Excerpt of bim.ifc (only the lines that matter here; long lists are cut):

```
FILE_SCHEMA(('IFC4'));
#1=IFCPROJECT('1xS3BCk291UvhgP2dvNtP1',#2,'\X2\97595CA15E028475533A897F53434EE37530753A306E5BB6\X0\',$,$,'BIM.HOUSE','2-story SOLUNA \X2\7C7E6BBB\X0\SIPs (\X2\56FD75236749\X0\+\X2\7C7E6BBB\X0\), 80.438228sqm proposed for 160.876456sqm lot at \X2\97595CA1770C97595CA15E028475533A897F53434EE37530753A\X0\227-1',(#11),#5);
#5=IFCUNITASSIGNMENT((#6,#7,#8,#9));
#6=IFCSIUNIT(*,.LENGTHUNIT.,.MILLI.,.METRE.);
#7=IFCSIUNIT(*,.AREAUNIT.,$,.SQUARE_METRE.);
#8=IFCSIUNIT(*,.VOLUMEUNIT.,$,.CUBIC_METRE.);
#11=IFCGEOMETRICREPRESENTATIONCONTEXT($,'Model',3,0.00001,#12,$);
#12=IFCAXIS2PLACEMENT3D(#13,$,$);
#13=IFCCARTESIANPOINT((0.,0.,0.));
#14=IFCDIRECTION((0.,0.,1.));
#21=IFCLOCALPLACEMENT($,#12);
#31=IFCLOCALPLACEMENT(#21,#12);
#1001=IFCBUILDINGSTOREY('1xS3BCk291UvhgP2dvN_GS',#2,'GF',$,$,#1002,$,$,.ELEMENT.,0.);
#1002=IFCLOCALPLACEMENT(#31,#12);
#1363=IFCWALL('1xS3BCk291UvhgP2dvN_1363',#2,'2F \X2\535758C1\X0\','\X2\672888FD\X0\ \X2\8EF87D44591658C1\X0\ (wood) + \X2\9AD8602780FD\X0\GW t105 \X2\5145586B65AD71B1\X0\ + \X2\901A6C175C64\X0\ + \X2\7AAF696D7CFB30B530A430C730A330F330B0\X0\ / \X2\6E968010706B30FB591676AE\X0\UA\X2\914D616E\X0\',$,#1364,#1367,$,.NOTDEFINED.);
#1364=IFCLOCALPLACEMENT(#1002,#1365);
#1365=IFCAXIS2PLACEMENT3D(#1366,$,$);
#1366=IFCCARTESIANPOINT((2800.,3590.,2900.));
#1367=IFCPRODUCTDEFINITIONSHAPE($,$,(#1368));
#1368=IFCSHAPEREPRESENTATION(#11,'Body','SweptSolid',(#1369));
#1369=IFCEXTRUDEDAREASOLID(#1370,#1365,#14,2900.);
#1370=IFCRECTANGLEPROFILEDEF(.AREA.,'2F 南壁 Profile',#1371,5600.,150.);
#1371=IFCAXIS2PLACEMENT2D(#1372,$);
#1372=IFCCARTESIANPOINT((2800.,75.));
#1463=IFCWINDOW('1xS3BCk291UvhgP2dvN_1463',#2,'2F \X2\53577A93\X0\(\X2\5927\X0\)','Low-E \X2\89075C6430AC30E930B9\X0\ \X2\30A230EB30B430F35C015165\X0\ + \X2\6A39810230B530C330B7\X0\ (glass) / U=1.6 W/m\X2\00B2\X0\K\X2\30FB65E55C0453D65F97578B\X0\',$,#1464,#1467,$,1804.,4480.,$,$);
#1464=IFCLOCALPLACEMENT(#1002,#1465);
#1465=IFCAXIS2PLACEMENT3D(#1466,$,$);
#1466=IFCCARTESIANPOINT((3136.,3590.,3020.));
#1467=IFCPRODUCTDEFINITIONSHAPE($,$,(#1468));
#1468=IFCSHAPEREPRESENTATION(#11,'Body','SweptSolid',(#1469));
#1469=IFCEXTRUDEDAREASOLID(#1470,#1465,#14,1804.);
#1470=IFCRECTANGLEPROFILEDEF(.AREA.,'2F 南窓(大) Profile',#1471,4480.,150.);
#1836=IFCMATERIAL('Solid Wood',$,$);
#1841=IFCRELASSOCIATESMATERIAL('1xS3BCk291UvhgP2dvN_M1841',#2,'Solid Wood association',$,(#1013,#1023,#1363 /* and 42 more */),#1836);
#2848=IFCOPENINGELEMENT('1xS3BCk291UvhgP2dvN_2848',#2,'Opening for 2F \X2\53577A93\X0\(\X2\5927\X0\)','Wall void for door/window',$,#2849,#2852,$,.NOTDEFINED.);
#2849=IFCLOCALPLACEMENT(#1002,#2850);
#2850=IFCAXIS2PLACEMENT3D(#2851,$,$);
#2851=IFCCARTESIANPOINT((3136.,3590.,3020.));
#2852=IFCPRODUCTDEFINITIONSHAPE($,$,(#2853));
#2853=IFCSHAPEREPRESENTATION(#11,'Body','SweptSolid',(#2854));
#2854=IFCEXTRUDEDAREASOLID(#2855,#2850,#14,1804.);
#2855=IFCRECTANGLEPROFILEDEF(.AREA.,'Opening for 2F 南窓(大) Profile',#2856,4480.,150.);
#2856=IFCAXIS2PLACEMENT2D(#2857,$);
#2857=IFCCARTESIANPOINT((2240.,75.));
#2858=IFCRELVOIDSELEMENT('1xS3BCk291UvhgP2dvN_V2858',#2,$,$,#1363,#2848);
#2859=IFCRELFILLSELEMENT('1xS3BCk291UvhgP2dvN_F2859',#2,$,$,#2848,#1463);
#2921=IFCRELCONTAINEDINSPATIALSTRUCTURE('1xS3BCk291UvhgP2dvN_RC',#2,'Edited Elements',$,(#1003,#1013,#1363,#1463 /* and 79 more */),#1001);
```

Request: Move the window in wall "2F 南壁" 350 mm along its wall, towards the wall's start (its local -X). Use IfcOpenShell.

```python
import ifcopenshell
import ifcopenshell.api.geometry
import ifcopenshell.util.placement

model = ifcopenshell.open("bim.ifc")

window = model.by_id(1463)
opening = window.FillsVoids[0].RelatingOpeningElement
wall = opening.VoidsElements[0].RelatingBuildingElement

wall_matrix = ifcopenshell.util.placement.get_local_placement(wall.ObjectPlacement)
shift = wall_matrix[:3, 0] * -350.0
before = ifcopenshell.util.placement.get_local_placement(window.ObjectPlacement)[:3, 3].copy()

# The window is not placed relative to its opening, so move both.
for product in (opening, window):
    matrix = ifcopenshell.util.placement.get_local_placement(product.ObjectPlacement)
    matrix[:3, 3] += shift
    ifcopenshell.api.geometry.edit_object_placement(model, product=product, matrix=matrix, is_si=False)

after = ifcopenshell.util.placement.get_local_placement(window.ObjectPlacement)[:3, 3]
print("window moved by", (after - before).round(3) + 0.0)

model.write("bim_rev.ifc")
```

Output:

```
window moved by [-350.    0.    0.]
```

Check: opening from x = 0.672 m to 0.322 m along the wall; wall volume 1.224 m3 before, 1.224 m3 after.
